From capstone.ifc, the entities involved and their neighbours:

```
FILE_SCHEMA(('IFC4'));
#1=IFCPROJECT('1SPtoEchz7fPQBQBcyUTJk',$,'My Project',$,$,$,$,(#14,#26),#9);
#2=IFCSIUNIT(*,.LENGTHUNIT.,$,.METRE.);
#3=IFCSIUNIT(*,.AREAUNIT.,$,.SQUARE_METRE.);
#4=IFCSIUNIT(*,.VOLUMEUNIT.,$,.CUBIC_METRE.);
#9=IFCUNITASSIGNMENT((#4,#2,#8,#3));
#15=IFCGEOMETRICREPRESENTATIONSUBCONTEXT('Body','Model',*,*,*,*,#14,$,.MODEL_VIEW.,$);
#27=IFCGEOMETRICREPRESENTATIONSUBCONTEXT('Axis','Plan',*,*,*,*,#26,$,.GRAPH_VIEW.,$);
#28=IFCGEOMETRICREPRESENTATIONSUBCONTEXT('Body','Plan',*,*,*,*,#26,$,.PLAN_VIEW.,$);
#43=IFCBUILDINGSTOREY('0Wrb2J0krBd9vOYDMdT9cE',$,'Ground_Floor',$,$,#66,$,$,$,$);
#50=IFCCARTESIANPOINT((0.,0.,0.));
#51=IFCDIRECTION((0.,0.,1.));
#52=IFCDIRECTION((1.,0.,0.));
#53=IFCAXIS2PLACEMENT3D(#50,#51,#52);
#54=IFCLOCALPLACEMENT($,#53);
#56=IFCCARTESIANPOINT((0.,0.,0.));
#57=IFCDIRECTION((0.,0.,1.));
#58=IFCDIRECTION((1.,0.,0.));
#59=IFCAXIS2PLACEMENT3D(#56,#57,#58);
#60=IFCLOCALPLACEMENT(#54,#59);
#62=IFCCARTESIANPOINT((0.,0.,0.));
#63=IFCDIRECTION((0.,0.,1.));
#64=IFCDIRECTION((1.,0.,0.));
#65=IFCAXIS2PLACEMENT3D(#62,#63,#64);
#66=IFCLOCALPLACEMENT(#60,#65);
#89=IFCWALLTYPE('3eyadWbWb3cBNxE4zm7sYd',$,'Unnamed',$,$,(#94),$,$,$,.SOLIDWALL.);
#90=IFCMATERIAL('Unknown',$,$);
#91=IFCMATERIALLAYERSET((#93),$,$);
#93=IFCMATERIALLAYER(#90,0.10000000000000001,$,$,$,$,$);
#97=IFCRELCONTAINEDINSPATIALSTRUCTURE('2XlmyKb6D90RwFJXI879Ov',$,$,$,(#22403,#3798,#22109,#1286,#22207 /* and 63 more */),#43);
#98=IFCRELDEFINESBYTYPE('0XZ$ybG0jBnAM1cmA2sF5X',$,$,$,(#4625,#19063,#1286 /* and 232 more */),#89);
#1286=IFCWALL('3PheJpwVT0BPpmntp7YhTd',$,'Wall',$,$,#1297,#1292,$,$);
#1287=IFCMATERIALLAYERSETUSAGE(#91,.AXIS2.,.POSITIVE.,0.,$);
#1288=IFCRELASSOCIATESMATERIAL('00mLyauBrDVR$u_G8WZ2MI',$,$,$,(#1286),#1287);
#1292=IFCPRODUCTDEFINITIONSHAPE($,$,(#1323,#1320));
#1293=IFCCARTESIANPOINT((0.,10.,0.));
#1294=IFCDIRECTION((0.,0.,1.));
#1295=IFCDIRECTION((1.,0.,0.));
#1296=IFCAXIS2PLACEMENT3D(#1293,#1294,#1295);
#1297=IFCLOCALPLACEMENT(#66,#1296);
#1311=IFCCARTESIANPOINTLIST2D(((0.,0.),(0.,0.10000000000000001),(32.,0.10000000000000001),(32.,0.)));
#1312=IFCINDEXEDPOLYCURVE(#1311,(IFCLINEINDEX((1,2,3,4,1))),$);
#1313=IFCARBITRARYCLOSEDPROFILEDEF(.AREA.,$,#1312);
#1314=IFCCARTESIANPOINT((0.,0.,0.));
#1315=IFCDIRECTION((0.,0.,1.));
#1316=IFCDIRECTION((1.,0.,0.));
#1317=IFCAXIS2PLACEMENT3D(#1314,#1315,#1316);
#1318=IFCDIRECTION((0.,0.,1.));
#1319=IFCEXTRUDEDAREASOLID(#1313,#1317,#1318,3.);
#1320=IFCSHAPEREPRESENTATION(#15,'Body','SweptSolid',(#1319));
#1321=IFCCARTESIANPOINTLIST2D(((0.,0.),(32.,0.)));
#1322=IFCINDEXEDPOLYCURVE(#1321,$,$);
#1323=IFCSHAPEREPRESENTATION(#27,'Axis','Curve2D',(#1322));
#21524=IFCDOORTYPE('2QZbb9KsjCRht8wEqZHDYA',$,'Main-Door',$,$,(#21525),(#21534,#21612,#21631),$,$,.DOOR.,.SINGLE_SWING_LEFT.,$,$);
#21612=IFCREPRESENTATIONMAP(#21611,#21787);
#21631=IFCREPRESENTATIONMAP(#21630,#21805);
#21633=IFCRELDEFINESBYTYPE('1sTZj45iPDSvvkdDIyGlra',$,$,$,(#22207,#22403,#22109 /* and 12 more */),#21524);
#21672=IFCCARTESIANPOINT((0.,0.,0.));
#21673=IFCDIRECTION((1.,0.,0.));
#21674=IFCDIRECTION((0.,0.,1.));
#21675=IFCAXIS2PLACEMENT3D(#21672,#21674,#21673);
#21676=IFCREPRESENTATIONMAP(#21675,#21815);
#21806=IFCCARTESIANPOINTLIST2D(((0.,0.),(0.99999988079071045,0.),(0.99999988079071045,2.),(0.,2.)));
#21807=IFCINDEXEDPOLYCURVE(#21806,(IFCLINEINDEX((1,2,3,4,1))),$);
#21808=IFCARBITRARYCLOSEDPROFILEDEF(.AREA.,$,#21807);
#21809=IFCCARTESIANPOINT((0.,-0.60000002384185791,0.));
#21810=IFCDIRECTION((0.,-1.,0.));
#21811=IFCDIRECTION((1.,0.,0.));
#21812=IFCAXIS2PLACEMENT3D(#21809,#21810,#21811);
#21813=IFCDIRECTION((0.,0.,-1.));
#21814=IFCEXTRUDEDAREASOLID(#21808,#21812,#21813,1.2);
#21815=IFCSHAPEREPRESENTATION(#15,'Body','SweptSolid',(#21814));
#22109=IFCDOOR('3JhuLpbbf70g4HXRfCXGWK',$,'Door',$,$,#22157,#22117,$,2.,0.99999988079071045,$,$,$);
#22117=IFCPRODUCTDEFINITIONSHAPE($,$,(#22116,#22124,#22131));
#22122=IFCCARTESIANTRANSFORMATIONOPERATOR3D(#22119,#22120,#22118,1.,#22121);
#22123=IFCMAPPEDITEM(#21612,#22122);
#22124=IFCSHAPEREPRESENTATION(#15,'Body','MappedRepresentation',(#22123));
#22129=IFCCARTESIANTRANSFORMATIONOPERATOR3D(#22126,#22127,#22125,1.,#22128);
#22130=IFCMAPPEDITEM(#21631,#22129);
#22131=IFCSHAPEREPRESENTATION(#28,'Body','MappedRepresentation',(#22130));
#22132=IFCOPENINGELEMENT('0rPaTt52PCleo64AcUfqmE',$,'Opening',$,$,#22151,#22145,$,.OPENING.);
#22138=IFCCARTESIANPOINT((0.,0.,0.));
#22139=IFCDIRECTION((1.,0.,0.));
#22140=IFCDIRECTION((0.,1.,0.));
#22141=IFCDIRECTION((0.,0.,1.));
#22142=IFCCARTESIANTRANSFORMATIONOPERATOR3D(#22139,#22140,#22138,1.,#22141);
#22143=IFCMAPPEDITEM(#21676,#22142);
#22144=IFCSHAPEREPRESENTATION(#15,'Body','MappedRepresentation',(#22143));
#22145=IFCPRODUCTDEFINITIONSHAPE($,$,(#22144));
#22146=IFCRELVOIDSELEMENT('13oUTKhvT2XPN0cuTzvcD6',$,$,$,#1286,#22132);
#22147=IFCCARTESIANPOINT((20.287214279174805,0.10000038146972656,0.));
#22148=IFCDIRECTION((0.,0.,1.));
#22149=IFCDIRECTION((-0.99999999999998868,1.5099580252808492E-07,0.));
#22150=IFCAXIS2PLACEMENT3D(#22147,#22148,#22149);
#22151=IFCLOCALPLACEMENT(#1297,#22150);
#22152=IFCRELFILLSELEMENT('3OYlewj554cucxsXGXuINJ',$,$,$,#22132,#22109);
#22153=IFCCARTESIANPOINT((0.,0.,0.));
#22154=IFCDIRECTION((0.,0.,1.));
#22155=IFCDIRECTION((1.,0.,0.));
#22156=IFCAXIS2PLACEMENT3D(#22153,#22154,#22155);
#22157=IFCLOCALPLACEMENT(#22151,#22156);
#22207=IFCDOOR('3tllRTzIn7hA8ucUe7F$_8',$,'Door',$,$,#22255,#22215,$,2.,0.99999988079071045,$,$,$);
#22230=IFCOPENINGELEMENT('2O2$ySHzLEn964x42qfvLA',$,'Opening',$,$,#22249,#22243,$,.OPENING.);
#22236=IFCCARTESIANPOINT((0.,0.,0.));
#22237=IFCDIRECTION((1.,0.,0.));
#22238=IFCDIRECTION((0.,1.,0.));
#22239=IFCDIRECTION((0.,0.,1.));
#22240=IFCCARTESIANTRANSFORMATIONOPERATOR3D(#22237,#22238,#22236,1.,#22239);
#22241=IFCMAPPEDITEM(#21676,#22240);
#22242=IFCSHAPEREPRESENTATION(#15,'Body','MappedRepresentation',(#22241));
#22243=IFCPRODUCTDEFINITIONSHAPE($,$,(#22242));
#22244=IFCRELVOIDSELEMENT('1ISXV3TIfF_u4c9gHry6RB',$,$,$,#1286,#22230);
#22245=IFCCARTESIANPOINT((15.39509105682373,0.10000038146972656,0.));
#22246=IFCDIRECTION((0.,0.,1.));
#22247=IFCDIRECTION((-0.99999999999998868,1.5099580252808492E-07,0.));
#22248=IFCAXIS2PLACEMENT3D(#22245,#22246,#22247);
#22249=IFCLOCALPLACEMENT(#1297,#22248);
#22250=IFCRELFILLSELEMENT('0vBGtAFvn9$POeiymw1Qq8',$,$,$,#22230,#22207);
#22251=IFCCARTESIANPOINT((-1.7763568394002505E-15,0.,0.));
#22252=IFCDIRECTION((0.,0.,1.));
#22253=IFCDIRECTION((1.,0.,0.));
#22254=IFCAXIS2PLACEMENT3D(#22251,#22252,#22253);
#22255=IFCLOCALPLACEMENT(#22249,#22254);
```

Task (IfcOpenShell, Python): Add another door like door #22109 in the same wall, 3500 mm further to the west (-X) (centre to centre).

```python
import ifcopenshell
import ifcopenshell.api.feature
import ifcopenshell.api.geometry
import ifcopenshell.api.root
import ifcopenshell.geom
import ifcopenshell.util.element
import ifcopenshell.util.placement
import ifcopenshell.util.shape
import ifcopenshell.util.unit

model = ifcopenshell.open("capstone.ifc")
unit_scale = ifcopenshell.util.unit.calculate_unit_scale(model)
settings = ifcopenshell.geom.settings()


def volume(element):
    """Net volume in cubic metres, openings subtracted."""
    shape = ifcopenshell.geom.create_shape(settings, element)
    return ifcopenshell.util.shape.get_volume(shape.geometry)


door = model.by_guid("3JhuLpbbf70g4HXRfCXGWK")
opening = door.FillsVoids[0].RelatingOpeningElement
wall = opening.VoidsElements[0].RelatingBuildingElement
before = volume(wall)
shift = ifcopenshell.util.placement.get_local_placement(wall.ObjectPlacement)[:3, 0] * -3.5 / unit_scale

# copy_class copies the void relationship, type, container and properties, but no geometry.
new_opening = ifcopenshell.api.root.copy_class(model, product=opening)
new_opening.Representation = ifcopenshell.util.element.copy_deep(
    model, opening.Representation, exclude=["IfcGeometricRepresentationContext", "IfcRepresentationMap"]
)
new_door = ifcopenshell.api.root.copy_class(model, product=door)
new_door.Representation = ifcopenshell.util.element.copy_deep(
    model, door.Representation, exclude=["IfcGeometricRepresentationContext", "IfcRepresentationMap"]
)
ifcopenshell.api.feature.add_filling(model, opening=new_opening, element=new_door)

for old, new in ((opening, new_opening), (door, new_door)):
    matrix = ifcopenshell.util.placement.get_local_placement(old.ObjectPlacement)
    matrix[:3, 3] += shift
    ifcopenshell.api.geometry.edit_object_placement(model, product=new, matrix=matrix, is_si=False)

after = volume(wall)

print(f"wall volume {before:.3f} -> {after:.3f} m3")

model.write("capstone_edited.ifc")
```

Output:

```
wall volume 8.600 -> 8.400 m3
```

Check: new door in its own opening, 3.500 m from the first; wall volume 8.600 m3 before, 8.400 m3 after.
